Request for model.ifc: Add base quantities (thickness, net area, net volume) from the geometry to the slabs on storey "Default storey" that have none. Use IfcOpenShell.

First a look at what the model holds.

```python
import ifcopenshell
import ifcopenshell.util.element
import ifcopenshell.util.unit

model = ifcopenshell.open("model.ifc")
print(model.schema)
for unit_type in ("LENGTHUNIT", "AREAUNIT", "VOLUMEUNIT"):
    print(unit_type, ifcopenshell.util.unit.calculate_unit_scale(model, unit_type))
storey = next(s for s in model.by_type("IfcBuildingStorey") if s.Name == "Default storey")
slabs = [e for e in ifcopenshell.util.element.get_decomposition(storey) if e.is_a("IfcSlab")]
for e in sorted(slabs, key=lambda e: e.id()):
    print(e.id(), e.is_a(), e.Name, list(ifcopenshell.util.element.get_psets(e, qtos_only=True)), sep=" | ")
```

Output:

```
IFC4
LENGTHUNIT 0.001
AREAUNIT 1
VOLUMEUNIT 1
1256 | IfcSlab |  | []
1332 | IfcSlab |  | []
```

```python
import ifcopenshell
import ifcopenshell.api.pset
import ifcopenshell.geom
import ifcopenshell.util.element
import ifcopenshell.util.shape
import ifcopenshell.util.unit

model = ifcopenshell.open("model.ifc")
unit_scale = ifcopenshell.util.unit.calculate_unit_scale(model)
area_scale = ifcopenshell.util.unit.calculate_unit_scale(model, "AREAUNIT")
volume_scale = ifcopenshell.util.unit.calculate_unit_scale(model, "VOLUMEUNIT")
settings = ifcopenshell.geom.settings()

storey = next(s for s in model.by_type("IfcBuildingStorey") if s.Name == "Default storey")
slabs = [e for e in ifcopenshell.util.element.get_decomposition(storey) if e.is_a("IfcSlab")]

for e in sorted(slabs, key=lambda e: e.id()):
    if ifcopenshell.util.element.get_psets(e, qtos_only=True, should_inherit=False):
        continue
    # Geometry comes back in metres, in the element's own axes.
    shape = ifcopenshell.geom.create_shape(settings, e)
    values = {
        "Width": ifcopenshell.util.shape.get_z(shape.geometry) / unit_scale,
        "NetArea": ifcopenshell.util.shape.get_footprint_area(shape.geometry) / area_scale,
        "NetVolume": ifcopenshell.util.shape.get_volume(shape.geometry) / volume_scale,
    }
    qto = ifcopenshell.api.pset.add_qto(model, product=e, name="Qto_SlabBaseQuantities")
    ifcopenshell.api.pset.edit_qto(model, qto=qto, properties=values)
    print(e.id(), {k: round(v, 3) for k, v in values.items()})

model.write("model_v2.ifc")
```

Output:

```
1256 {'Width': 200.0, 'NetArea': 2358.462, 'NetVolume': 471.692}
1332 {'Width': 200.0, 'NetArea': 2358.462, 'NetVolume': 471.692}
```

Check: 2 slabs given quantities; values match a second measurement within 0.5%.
